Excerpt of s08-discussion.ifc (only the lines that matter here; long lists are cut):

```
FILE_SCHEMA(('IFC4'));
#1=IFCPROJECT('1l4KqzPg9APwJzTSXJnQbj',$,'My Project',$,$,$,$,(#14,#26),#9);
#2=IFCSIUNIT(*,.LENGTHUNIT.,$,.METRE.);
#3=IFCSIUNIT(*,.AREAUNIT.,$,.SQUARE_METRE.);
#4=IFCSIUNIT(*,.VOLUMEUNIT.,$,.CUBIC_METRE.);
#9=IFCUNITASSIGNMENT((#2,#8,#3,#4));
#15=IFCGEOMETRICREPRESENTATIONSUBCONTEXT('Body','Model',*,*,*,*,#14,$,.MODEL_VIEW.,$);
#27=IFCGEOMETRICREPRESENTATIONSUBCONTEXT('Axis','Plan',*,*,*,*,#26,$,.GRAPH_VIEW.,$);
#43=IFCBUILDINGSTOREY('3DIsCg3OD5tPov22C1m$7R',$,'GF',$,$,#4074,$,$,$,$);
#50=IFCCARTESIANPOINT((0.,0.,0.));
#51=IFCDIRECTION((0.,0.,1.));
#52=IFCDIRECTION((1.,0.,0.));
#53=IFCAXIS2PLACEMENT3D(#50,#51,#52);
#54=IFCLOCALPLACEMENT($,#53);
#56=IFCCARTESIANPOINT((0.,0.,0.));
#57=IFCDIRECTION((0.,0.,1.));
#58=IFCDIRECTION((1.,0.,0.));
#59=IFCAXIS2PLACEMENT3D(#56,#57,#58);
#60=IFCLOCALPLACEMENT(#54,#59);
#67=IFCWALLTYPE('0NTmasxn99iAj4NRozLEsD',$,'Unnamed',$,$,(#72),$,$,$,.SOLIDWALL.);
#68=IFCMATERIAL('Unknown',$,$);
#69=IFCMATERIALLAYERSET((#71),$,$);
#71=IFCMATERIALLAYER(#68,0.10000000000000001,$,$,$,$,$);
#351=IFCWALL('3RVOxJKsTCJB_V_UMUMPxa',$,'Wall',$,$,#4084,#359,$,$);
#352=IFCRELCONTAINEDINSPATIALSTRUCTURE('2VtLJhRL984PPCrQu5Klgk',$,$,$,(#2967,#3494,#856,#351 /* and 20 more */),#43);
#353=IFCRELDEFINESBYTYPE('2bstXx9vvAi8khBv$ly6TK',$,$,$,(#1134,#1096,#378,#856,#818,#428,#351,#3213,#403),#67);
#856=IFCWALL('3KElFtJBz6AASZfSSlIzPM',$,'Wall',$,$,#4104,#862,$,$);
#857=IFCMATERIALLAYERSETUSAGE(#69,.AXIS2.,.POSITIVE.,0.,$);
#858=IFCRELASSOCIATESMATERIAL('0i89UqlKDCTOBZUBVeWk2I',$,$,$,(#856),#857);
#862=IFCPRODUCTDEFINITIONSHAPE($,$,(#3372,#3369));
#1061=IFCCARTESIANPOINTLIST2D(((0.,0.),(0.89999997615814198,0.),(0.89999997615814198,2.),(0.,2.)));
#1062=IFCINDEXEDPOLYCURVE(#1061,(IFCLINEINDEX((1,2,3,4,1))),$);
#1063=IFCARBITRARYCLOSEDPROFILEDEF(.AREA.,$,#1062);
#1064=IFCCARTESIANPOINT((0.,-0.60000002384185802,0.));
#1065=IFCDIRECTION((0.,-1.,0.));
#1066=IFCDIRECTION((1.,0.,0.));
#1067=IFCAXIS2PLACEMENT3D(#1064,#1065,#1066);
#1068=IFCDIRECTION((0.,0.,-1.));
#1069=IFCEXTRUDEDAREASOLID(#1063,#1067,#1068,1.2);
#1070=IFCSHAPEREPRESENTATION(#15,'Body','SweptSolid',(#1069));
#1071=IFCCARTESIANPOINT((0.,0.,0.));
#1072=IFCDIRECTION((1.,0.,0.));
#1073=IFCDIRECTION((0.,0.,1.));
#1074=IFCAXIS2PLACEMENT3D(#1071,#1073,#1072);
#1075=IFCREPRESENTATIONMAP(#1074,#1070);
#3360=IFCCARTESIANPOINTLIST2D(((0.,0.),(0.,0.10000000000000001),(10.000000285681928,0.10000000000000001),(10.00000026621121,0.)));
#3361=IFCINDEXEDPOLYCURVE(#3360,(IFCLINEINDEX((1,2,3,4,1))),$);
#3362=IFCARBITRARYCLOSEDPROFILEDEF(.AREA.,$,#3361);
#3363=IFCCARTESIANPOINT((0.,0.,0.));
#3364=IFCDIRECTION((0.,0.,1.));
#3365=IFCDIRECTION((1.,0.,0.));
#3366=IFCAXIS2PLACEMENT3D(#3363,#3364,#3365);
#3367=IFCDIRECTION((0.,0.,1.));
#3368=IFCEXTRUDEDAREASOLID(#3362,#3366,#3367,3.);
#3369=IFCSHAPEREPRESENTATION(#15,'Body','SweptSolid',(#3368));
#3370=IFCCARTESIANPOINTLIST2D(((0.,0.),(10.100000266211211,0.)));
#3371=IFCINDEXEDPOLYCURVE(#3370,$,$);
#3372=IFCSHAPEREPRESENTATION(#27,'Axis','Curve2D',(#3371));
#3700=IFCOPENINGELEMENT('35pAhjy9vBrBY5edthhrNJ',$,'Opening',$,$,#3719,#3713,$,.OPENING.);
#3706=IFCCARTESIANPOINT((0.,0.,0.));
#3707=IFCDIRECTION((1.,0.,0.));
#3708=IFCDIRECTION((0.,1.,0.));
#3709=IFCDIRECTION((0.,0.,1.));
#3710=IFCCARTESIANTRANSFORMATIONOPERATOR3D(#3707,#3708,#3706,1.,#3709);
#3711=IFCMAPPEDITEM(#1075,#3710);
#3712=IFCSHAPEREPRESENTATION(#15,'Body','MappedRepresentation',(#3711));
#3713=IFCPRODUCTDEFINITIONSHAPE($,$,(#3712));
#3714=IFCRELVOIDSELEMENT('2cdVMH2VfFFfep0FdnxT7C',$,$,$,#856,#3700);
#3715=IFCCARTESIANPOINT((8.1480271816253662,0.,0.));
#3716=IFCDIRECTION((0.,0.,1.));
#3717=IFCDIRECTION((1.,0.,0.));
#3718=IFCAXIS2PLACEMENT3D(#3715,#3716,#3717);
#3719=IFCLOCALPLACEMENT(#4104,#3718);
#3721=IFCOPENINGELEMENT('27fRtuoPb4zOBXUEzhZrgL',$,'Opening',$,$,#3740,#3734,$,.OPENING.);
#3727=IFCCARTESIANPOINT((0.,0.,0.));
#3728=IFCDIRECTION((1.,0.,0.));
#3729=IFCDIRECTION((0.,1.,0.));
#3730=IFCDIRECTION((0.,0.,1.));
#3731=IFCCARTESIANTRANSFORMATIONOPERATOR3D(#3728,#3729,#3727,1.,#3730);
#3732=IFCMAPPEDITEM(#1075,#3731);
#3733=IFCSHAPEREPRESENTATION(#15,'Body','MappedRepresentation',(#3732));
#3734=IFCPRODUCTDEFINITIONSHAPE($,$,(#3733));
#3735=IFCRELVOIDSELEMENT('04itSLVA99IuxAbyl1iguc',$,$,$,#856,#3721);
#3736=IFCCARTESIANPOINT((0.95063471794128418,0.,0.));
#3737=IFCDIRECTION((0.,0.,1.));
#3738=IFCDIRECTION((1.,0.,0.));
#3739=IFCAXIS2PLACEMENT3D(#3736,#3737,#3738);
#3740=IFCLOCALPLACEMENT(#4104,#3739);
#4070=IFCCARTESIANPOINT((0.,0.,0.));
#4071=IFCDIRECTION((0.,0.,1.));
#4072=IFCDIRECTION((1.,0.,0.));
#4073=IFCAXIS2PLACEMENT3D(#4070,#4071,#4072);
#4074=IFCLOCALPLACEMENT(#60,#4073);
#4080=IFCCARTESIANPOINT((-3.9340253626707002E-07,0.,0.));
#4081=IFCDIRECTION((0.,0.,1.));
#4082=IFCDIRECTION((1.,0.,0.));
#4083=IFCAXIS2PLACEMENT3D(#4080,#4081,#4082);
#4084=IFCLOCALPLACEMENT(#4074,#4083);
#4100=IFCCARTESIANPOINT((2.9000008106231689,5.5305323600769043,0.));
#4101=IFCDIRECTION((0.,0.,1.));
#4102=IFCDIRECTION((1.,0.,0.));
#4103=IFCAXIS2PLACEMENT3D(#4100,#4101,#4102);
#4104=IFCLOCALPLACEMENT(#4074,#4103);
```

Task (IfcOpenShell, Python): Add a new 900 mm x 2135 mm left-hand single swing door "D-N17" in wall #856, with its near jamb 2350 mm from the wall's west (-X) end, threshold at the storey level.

```python
import numpy as np
import ifcopenshell
import ifcopenshell.api.feature
import ifcopenshell.api.geometry
import ifcopenshell.api.root
import ifcopenshell.api.spatial
import ifcopenshell.geom
import ifcopenshell.util.element
import ifcopenshell.util.placement
import ifcopenshell.util.representation
import ifcopenshell.util.shape
import ifcopenshell.util.unit

model = ifcopenshell.open("s08-discussion.ifc")
unit_scale = ifcopenshell.util.unit.calculate_unit_scale(model)
settings = ifcopenshell.geom.settings()


def volume(element):
    """Net volume in cubic metres, openings subtracted."""
    shape = ifcopenshell.geom.create_shape(settings, element)
    return ifcopenshell.util.shape.get_volume(shape.geometry)


wall = model.by_guid("3KElFtJBz6AASZfSSlIzPM")
storey = ifcopenshell.util.element.get_container(wall, ifc_class="IfcBuildingStorey")
context = ifcopenshell.util.representation.get_context(model, "Model", "Body", "MODEL_VIEW")
before = volume(wall)

width, height, from_end, sill = 0.9, 2.135, 2.35, 0.0  # metres

# The wall runs along its own X axis, and the end named is its -X end.
wall_shape = ifcopenshell.geom.create_shape(settings, wall)
x, y, z = ifcopenshell.util.shape.get_vertices(wall_shape.geometry).T
start = x.min() + from_end
face, thickness = float(y.min()), float(y.max() - y.min())
wall_matrix = ifcopenshell.util.placement.get_local_placement(wall.ObjectPlacement)
level = ifcopenshell.util.placement.get_local_placement(storey.ObjectPlacement)[2, 3]


def in_wall(x, y):
    """Placement at x, y metres in the wall's axes, at sill height."""
    matrix = wall_matrix.copy()
    matrix[:, 3] = wall_matrix @ np.array([x / unit_scale, y / unit_scale, 0.0, 1.0])
    matrix[2, 3] = level + sill / unit_scale
    return matrix


# Opening: a box that overshoots both wall faces by 50 mm.
opening = ifcopenshell.api.root.create_entity(model, ifc_class="IfcOpeningElement", predefined_type="OPENING")
box = ifcopenshell.api.geometry.add_wall_representation(
    model, context=context, length=width, height=height, thickness=thickness + 0.1
)
ifcopenshell.api.geometry.assign_representation(model, product=opening, representation=box)
ifcopenshell.api.geometry.edit_object_placement(model, product=opening, matrix=in_wall(start, face - 0.05), is_si=False)
ifcopenshell.api.feature.add_feature(model, feature=opening, element=wall)

door = ifcopenshell.api.root.create_entity(model, ifc_class="IfcDoor", name="D-N17", predefined_type="DOOR")
door.OverallWidth, door.OverallHeight = width / unit_scale, height / unit_scale
door.OperationType = "SINGLE_SWING_LEFT"
body = ifcopenshell.api.geometry.add_door_representation(
    model,
    context=context,
    overall_width=door.OverallWidth,
    overall_height=door.OverallHeight,
    operation_type="SINGLE_SWING_LEFT",
    lining_properties={"LiningDepth": thickness / unit_scale, "ThresholdDepth": thickness / unit_scale},
)
ifcopenshell.api.geometry.assign_representation(model, product=door, representation=body)
ifcopenshell.api.spatial.assign_container(model, products=[door], relating_structure=storey)
ifcopenshell.api.feature.add_filling(model, opening=opening, element=door)

# The lining spans the wall, so the door starts at the wall face.
ifcopenshell.api.geometry.edit_object_placement(model, product=door, matrix=in_wall(start, face), is_si=False)

after = volume(wall)

print(f"wall volume {before:.3f} -> {after:.3f} m3")

model.write("s08-discussion_updated.ifc")
```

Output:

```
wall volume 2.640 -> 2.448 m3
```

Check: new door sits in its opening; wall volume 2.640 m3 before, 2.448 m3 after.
